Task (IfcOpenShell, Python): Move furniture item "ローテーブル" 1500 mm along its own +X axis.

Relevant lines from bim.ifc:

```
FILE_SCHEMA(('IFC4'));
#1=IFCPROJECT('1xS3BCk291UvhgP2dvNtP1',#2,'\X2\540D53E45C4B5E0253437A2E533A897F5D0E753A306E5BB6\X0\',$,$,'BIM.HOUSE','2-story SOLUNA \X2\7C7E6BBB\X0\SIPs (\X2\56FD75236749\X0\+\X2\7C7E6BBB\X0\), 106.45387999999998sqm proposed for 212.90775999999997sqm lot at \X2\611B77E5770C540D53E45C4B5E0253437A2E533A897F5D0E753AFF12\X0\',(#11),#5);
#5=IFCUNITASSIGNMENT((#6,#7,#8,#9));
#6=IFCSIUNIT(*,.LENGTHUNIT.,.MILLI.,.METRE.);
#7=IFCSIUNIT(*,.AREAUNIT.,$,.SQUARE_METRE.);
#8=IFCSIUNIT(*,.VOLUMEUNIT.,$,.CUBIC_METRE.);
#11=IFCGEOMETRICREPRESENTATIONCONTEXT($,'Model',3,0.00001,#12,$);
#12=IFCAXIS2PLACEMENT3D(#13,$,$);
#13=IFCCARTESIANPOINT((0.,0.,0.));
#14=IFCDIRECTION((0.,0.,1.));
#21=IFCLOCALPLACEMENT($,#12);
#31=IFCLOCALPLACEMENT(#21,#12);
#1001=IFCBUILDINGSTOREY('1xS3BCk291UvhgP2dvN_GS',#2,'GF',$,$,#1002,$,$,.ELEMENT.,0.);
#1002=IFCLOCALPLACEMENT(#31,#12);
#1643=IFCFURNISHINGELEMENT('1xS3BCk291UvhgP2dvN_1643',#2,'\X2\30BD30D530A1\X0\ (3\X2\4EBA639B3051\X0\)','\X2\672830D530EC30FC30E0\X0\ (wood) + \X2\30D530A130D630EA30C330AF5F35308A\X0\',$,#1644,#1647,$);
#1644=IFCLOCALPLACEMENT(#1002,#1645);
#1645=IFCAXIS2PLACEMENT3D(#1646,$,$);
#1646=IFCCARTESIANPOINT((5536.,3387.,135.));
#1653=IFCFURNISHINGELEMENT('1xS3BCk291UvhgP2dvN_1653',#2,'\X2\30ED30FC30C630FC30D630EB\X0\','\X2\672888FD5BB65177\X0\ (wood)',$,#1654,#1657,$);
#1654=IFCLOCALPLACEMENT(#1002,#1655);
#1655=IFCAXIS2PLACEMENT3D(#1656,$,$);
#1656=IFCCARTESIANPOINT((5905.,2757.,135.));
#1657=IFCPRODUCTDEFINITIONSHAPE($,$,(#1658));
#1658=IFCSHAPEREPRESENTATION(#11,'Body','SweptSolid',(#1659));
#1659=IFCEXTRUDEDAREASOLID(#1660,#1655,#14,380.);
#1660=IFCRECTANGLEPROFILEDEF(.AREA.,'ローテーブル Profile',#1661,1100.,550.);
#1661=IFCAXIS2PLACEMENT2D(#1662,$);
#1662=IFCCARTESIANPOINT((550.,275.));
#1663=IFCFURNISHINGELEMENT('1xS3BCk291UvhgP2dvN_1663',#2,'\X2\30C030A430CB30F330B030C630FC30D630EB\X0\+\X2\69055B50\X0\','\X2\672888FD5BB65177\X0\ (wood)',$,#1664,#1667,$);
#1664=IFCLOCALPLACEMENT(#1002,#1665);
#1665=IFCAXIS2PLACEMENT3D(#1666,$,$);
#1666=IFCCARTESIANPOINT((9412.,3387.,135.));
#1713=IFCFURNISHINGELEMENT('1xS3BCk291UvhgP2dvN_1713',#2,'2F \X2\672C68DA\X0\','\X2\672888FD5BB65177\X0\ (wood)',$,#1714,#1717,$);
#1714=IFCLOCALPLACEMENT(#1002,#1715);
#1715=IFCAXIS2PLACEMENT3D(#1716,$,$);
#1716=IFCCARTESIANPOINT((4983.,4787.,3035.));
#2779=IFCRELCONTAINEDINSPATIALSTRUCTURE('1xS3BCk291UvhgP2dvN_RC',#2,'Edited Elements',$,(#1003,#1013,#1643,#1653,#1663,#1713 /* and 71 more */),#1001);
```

```python
import ifcopenshell
import ifcopenshell.api.geometry
import ifcopenshell.util.placement

model = ifcopenshell.open("bim.ifc")

item = model.by_guid("1xS3BCk291UvhgP2dvN_1653")
matrix = ifcopenshell.util.placement.get_local_placement(item.ObjectPlacement)
matrix[:3, 3] += matrix[:3, 0] * 1500.0
ifcopenshell.api.geometry.edit_object_placement(model, product=item, matrix=matrix, is_si=False)

print(ifcopenshell.util.placement.get_local_placement(item.ObjectPlacement).round(3) + 0.0)

model.write("bim_updated.ifc")
```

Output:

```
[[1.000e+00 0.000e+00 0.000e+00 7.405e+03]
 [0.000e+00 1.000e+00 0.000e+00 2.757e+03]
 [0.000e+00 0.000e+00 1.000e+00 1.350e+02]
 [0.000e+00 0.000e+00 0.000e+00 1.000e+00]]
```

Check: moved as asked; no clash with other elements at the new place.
